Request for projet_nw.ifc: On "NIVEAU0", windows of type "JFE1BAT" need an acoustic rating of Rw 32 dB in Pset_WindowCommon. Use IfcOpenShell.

First a look at what the model holds.

```python
import ifcopenshell
import ifcopenshell.util.element

model = ifcopenshell.open("projet_nw.ifc")
print(model.schema)
storey = next(s for s in model.by_type("IfcBuildingStorey") if s.Name == "NIVEAU0")
windows = [e for e in ifcopenshell.util.element.get_decomposition(storey) if e.is_a("IfcWindow")]
seen = {}
for e in windows:
    element_type = ifcopenshell.util.element.get_type(e)
    key = (element_type.Name if element_type != e and element_type else None, ifcopenshell.util.element.get_pset(e, "Pset_WindowCommon", "AcousticRating"))
    seen[key] = seen.get(key, 0) + 1
for (name, value), count in sorted(seen.items(), key=str):
    print(count, "x", name, "|", value)
```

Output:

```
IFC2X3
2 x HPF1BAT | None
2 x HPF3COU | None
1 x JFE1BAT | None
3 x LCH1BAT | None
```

```python
import ifcopenshell
import ifcopenshell.api.pset
import ifcopenshell.util.element

model = ifcopenshell.open("projet_nw.ifc")

storey = next(s for s in model.by_type("IfcBuildingStorey") if s.Name == "NIVEAU0")
windows = [e for e in ifcopenshell.util.element.get_decomposition(storey) if e.is_a("IfcWindow")]

count = 0
for e in windows:
    element_type = ifcopenshell.util.element.get_type(e)
    if element_type in (None, e) or element_type.Name != "JFE1BAT":
        continue
    # add_pset returns the element's existing set when there is one.
    pset = ifcopenshell.api.pset.add_pset(model, product=e, name="Pset_WindowCommon")
    ifcopenshell.api.pset.edit_pset(model, pset=pset, properties={"AcousticRating": "Rw 32 dB"})
    count += 1

print(count, "windows updated")

model.write("projet_nw_v2.ifc")
```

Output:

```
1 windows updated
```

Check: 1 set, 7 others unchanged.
